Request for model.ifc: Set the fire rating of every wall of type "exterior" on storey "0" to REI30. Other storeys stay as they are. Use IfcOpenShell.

First a look at what the model holds.

```python
import ifcopenshell
import ifcopenshell.util.element

model = ifcopenshell.open("model.ifc")
print(model.schema)
storey = next(s for s in model.by_type("IfcBuildingStorey") if s.Name == "0")
walls = [e for e in ifcopenshell.util.element.get_decomposition(storey) if e.is_a("IfcWall")]
seen = {}
for e in walls:
    element_type = ifcopenshell.util.element.get_type(e)
    key = (element_type.Name if element_type != e and element_type else None, ifcopenshell.util.element.get_pset(e, "Pset_WallCommon", "FireRating"))
    seen[key] = seen.get(key, 0) + 1
for (name, value), count in sorted(seen.items(), key=str):
    print(count, "x", name, "|", value)
```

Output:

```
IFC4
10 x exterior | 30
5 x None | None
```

```python
import ifcopenshell
import ifcopenshell.api.pset
import ifcopenshell.util.element

model = ifcopenshell.open("model.ifc")

storey = next(s for s in model.by_type("IfcBuildingStorey") if s.Name == "0")
walls = [e for e in ifcopenshell.util.element.get_decomposition(storey) if e.is_a("IfcWall")]

count = 0
for e in walls:
    element_type = ifcopenshell.util.element.get_type(e)
    if element_type in (None, e) or element_type.Name != "exterior":
        continue
    # add_pset returns the element's existing set when there is one.
    pset = ifcopenshell.api.pset.add_pset(model, product=e, name="Pset_WallCommon")
    ifcopenshell.api.pset.edit_pset(model, pset=pset, properties={"FireRating": "REI30"})
    count += 1

print(count, "walls updated")

model.write("model_edited.ifc")
```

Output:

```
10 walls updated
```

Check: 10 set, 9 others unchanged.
